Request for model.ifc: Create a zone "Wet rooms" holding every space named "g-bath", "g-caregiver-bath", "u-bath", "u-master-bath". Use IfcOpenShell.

First a look at what the model holds.

```python
import ifcopenshell

model = ifcopenshell.open("model.ifc")
print(model.schema)
seen = {}
for space in model.by_type("IfcSpace"):
    seen[space.LongName] = seen.get(space.LongName, 0) + 1
for name, count in sorted(seen.items(), key=str):
    print(count, "x", name)
print("zones:", [z.Name for z in model.by_type("IfcZone")][:20])
```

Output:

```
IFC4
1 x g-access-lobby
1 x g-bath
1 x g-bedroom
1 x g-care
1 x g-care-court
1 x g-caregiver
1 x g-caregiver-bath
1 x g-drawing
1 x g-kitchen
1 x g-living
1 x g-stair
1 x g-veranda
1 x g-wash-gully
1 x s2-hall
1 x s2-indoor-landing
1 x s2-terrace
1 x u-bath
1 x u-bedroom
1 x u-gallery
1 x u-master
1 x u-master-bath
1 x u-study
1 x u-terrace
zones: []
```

```python
import ifcopenshell
import ifcopenshell.api.group
import ifcopenshell.api.root

model = ifcopenshell.open("model.ifc")

names = {"g-bath", "g-caregiver-bath", "u-bath", "u-master-bath"}
spaces = [s for s in model.by_type("IfcSpace") if s.LongName in names]

zone = ifcopenshell.api.root.create_entity(model, ifc_class="IfcZone", name="Wet rooms")
ifcopenshell.api.group.assign_group(model, products=spaces, group=zone)
print(len(spaces), "spaces in", zone.Name)

model.write("model_edited.ifc")
```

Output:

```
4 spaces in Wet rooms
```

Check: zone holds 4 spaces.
